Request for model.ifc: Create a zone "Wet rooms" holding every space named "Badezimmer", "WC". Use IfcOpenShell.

First a look at what the model holds.

```python
import ifcopenshell

model = ifcopenshell.open("model.ifc")
print(model.schema)
seen = {}
for space in model.by_type("IfcSpace"):
    seen[space.LongName] = seen.get(space.LongName, 0) + 1
for name, count in sorted(seen.items(), key=str):
    print(count, "x", name)
print("zones:", [z.Name for z in model.by_type("IfcZone")][:20])
```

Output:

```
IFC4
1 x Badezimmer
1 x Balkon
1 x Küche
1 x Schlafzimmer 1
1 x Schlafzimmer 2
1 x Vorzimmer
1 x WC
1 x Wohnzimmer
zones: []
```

```python
import ifcopenshell
import ifcopenshell.api.group
import ifcopenshell.api.root

model = ifcopenshell.open("model.ifc")

names = {"Badezimmer", "WC"}
spaces = [s for s in model.by_type("IfcSpace") if s.LongName in names]

zone = ifcopenshell.api.root.create_entity(model, ifc_class="IfcZone", name="Wet rooms")
ifcopenshell.api.group.assign_group(model, products=spaces, group=zone)
print(len(spaces), "spaces in", zone.Name)

model.write("model_rev.ifc")
```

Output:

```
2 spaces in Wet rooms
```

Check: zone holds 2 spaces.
